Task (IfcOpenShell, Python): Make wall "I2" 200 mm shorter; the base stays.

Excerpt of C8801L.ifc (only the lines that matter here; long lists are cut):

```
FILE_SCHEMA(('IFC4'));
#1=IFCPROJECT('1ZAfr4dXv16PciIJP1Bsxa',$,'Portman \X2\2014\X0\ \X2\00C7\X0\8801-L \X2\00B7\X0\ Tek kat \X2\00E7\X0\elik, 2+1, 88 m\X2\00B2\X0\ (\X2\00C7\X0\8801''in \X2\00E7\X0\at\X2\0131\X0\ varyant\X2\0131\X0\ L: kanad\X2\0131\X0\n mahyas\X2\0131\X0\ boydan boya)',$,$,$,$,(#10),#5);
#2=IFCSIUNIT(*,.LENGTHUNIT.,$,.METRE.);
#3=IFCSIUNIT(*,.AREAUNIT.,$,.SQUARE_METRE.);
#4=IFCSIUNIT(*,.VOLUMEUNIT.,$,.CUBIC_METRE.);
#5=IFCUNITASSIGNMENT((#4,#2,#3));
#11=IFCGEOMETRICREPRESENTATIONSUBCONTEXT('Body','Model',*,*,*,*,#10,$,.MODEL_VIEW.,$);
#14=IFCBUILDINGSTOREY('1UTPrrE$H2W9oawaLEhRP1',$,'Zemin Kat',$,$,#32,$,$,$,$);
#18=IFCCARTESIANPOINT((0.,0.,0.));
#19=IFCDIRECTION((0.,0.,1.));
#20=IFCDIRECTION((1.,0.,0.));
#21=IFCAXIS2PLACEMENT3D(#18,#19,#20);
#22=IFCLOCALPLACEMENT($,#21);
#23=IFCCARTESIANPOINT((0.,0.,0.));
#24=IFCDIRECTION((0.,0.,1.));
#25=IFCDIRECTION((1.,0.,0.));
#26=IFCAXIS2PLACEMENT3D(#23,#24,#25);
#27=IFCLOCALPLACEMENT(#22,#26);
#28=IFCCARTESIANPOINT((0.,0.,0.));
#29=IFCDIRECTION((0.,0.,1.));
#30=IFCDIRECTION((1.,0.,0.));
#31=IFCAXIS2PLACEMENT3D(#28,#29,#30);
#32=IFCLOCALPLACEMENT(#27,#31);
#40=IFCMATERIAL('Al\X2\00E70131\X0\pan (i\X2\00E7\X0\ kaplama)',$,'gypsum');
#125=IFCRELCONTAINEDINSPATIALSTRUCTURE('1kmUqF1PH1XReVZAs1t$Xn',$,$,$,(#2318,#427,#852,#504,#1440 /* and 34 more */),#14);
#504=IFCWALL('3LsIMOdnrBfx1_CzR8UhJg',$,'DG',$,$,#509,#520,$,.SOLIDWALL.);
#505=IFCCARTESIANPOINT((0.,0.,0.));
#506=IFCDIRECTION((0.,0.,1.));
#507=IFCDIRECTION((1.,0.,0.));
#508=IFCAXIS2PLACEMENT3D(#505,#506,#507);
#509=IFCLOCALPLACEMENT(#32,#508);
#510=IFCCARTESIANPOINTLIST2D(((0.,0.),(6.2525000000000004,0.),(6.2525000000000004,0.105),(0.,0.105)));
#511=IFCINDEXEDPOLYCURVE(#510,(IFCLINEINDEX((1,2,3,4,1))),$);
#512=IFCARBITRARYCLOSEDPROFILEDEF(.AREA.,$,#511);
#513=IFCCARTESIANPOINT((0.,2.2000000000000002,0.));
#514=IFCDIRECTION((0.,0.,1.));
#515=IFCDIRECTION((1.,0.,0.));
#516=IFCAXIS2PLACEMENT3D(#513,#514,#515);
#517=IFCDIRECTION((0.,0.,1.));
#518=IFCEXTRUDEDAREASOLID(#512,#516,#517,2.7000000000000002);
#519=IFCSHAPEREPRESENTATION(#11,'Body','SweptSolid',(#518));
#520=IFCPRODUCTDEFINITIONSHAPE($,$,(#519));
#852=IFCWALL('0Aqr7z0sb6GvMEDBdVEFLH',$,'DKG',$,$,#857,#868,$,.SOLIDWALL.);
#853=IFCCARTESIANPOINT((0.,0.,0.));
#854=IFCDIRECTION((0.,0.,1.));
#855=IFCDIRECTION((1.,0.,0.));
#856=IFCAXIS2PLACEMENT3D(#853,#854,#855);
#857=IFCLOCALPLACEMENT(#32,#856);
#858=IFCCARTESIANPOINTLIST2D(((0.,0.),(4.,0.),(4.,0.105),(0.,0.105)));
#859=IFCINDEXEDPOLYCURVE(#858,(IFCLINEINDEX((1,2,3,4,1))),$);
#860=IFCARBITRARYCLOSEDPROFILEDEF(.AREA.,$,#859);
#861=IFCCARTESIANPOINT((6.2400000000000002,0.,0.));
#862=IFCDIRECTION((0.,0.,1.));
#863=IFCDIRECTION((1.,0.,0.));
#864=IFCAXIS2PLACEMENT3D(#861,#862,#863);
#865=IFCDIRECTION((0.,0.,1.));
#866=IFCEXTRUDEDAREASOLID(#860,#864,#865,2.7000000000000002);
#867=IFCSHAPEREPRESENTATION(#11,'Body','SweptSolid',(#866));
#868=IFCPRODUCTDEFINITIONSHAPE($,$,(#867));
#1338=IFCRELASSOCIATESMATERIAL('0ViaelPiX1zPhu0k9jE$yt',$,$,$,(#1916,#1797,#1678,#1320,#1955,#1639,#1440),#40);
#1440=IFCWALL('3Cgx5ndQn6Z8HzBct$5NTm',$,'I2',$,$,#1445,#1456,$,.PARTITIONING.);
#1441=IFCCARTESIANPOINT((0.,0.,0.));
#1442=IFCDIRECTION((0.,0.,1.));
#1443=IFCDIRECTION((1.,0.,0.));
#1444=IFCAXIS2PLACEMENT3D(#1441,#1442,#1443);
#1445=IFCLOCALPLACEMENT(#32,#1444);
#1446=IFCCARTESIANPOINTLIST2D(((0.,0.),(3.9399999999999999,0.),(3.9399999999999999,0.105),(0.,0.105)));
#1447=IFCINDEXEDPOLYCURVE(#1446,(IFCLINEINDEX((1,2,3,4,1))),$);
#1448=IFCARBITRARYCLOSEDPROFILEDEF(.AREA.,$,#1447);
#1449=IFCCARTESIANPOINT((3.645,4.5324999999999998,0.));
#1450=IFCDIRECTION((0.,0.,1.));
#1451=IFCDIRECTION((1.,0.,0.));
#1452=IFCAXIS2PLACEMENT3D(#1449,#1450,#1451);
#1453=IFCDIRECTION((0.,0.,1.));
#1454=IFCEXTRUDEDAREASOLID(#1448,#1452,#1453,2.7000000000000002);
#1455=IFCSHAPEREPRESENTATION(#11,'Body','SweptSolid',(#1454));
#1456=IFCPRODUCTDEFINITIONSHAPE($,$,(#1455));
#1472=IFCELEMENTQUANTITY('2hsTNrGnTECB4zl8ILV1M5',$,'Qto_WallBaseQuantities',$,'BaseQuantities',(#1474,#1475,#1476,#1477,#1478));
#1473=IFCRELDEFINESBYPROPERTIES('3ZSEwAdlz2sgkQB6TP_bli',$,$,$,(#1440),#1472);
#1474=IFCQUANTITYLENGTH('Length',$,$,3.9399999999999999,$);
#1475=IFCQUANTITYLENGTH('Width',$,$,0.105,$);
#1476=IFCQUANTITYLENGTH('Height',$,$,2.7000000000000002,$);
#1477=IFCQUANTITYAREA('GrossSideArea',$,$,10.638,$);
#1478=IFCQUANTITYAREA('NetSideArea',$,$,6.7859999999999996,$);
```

```python
import ifcopenshell
import ifcopenshell.api.pset
import ifcopenshell.geom
import ifcopenshell.util.element
import ifcopenshell.util.representation
import ifcopenshell.util.shape
import ifcopenshell.util.unit

model = ifcopenshell.open("C8801L.ifc")
unit_scale = ifcopenshell.util.unit.calculate_unit_scale(model)
area_scale = ifcopenshell.util.unit.calculate_unit_scale(model, "AREAUNIT")
settings = ifcopenshell.geom.settings()


def volume(element):
    """Net volume in cubic metres, openings subtracted."""
    shape = ifcopenshell.geom.create_shape(settings, element)
    return ifcopenshell.util.shape.get_volume(shape.geometry)


wall = model.by_guid("3Cgx5ndQn6Z8HzBct$5NTm")
before = volume(wall)

body = ifcopenshell.util.representation.get_representation(wall, "Model", "Body")
solid = body.Items[0]
old_height = solid.Depth
solid.Depth -= 0.2 / unit_scale
after = volume(wall)
thickness = 0.105  # wall thickness in metres

# Update the stored height, areas and volumes.
qto = model.by_id(ifcopenshell.util.element.get_pset(wall, "Qto_WallBaseQuantities", should_inherit=False)["id"])
ifcopenshell.api.pset.edit_qto(model, qto=qto, properties={
    "Height": solid.Depth,
    "GrossSideArea": ifcopenshell.util.element.get_pset(wall, "Qto_WallBaseQuantities", "GrossSideArea") * solid.Depth / old_height,
    "NetSideArea": after / thickness / area_scale,
})

print(f"height {old_height:g} -> {solid.Depth:g}, volume {before:.3f} -> {after:.3f} m3")

model.write("C8801L_updated.ifc")
```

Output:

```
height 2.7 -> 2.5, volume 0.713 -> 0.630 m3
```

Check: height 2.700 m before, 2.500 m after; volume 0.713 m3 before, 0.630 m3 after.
